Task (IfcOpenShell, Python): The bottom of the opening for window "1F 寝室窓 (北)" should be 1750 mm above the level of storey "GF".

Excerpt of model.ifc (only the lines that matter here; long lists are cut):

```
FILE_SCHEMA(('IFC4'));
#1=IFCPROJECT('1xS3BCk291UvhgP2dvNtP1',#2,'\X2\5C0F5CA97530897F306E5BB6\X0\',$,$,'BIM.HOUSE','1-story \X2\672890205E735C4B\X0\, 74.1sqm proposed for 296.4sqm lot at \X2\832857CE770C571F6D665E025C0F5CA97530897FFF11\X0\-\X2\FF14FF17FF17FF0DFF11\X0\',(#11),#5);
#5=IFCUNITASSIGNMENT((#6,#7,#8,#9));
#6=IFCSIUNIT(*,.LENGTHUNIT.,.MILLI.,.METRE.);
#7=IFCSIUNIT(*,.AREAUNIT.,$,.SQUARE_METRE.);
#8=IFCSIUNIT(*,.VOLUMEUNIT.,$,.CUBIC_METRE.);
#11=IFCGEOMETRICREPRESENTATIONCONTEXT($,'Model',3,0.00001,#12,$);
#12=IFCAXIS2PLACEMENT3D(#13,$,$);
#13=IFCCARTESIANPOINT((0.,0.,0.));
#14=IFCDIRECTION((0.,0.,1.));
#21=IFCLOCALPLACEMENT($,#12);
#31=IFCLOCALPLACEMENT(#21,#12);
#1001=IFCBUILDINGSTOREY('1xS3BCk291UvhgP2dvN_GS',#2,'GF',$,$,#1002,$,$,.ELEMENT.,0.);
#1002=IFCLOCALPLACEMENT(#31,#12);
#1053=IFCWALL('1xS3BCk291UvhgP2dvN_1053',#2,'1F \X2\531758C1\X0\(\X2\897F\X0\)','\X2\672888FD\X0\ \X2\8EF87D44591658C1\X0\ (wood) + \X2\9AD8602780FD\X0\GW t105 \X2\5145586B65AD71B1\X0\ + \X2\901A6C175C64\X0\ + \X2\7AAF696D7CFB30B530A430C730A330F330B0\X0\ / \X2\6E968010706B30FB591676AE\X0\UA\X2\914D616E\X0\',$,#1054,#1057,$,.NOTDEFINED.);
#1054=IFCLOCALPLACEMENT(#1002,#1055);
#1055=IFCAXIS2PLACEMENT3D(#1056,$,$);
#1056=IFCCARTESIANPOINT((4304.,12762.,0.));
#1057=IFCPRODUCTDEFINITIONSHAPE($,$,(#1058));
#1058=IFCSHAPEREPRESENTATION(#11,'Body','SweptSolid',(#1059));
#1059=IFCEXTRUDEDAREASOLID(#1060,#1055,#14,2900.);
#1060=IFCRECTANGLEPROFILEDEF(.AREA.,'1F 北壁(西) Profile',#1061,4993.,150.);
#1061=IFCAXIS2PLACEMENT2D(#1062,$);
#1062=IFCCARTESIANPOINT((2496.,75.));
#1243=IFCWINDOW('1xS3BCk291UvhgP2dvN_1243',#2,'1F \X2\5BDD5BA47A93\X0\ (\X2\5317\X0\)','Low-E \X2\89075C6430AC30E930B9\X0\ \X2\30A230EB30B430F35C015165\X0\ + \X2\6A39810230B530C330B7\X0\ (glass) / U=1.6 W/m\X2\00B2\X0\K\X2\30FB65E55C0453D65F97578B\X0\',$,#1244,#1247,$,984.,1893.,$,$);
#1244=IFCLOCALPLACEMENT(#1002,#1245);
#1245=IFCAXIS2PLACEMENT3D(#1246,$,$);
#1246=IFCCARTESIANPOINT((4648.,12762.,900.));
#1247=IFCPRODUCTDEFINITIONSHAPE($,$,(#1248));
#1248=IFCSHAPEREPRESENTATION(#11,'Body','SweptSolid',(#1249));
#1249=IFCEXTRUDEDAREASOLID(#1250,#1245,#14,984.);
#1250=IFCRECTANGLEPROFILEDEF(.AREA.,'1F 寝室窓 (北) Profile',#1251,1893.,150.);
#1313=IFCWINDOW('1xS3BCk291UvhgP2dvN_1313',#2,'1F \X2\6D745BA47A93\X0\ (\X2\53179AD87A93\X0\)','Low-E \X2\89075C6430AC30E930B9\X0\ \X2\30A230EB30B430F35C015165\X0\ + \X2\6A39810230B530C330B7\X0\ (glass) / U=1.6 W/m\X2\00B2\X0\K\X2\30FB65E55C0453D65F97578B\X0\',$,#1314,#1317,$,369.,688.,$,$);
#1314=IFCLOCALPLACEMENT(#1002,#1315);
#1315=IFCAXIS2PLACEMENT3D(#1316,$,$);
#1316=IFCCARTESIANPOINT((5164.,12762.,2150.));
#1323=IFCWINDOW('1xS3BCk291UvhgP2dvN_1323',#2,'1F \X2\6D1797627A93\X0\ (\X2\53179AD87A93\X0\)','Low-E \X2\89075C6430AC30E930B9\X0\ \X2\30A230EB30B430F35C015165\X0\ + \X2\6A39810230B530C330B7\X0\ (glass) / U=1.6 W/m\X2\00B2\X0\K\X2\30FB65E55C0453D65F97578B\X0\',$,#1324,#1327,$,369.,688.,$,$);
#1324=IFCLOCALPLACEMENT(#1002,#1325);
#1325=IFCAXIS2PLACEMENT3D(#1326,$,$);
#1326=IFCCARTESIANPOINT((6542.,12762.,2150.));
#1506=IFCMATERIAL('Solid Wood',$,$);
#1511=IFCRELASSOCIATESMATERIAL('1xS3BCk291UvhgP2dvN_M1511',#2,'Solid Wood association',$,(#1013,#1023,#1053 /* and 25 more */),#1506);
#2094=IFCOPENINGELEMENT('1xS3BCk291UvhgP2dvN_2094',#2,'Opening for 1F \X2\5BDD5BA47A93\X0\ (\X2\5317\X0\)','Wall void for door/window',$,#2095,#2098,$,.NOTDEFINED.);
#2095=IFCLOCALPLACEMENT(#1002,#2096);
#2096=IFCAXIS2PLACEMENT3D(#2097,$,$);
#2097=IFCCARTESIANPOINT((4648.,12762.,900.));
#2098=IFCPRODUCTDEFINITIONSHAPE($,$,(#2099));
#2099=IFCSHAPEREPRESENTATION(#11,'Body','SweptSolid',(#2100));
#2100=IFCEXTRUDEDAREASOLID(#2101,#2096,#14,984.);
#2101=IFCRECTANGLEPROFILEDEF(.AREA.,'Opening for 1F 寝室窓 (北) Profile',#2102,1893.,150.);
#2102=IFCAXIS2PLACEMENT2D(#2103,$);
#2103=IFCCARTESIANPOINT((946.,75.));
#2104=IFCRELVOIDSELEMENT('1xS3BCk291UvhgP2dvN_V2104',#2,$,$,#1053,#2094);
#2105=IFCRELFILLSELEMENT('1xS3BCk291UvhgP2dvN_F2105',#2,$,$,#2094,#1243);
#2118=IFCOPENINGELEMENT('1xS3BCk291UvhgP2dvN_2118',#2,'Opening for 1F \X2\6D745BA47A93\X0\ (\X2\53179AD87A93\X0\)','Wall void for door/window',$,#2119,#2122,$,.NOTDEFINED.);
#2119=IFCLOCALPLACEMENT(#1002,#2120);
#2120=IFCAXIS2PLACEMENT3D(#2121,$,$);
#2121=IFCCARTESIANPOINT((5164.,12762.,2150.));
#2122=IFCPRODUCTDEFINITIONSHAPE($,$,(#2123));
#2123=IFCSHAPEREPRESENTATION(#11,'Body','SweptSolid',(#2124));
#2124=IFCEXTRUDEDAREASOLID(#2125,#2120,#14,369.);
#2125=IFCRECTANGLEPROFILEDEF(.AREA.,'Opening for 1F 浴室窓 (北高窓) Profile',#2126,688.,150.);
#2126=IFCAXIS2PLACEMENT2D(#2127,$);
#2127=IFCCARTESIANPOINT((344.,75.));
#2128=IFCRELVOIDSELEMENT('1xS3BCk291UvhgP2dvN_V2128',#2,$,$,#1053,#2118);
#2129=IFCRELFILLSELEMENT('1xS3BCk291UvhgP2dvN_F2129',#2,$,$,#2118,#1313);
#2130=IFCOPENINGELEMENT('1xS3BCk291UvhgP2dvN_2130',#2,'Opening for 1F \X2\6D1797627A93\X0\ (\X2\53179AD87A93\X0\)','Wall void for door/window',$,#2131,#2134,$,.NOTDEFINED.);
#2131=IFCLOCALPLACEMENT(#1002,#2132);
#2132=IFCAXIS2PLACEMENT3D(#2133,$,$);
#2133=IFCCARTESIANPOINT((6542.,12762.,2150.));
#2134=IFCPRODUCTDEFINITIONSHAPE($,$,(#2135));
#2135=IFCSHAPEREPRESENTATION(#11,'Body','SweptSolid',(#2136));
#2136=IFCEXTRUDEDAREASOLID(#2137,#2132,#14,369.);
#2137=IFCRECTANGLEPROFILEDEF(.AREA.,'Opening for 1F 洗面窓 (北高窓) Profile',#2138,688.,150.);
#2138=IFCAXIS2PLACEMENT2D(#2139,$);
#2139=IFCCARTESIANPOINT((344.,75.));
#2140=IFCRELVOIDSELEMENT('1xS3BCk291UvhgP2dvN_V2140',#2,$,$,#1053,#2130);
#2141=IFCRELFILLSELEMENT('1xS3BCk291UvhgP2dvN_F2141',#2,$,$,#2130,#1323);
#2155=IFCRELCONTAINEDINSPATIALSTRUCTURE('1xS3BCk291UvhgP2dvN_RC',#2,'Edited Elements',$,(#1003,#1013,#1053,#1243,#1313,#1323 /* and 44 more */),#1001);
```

```python
import numpy as np
import ifcopenshell
import ifcopenshell.api.geometry
import ifcopenshell.geom
import ifcopenshell.util.element
import ifcopenshell.util.placement
import ifcopenshell.util.shape
import ifcopenshell.util.unit

model = ifcopenshell.open("model.ifc")
unit_scale = ifcopenshell.util.unit.calculate_unit_scale(model)

window = model.by_id(1243)
opening = window.FillsVoids[0].RelatingOpeningElement
storey = ifcopenshell.util.element.get_container(window, ifc_class="IfcBuildingStorey")
level = ifcopenshell.util.placement.get_local_placement(storey.ObjectPlacement)[2, 3]

# The opening's origin need not be at the sill, so measure its lowest point.
shape = ifcopenshell.geom.create_shape(ifcopenshell.geom.settings(), opening)
bottom = ifcopenshell.util.shape.get_shape_bottom_elevation(shape, shape.geometry) / unit_scale
dz = level + 1750.0 - bottom

shift = np.array([0.0, 0.0, dz])
# The window is not placed relative to its opening, so move both.
for product in (opening, window):
    matrix = ifcopenshell.util.placement.get_local_placement(product.ObjectPlacement)
    matrix[:3, 3] += shift
    ifcopenshell.api.geometry.edit_object_placement(model, product=product, matrix=matrix, is_si=False)

print(f"moved by {dz * unit_scale:+.3f} m")

model.write("model_updated.ifc")
```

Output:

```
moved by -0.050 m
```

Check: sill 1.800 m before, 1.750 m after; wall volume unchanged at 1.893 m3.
